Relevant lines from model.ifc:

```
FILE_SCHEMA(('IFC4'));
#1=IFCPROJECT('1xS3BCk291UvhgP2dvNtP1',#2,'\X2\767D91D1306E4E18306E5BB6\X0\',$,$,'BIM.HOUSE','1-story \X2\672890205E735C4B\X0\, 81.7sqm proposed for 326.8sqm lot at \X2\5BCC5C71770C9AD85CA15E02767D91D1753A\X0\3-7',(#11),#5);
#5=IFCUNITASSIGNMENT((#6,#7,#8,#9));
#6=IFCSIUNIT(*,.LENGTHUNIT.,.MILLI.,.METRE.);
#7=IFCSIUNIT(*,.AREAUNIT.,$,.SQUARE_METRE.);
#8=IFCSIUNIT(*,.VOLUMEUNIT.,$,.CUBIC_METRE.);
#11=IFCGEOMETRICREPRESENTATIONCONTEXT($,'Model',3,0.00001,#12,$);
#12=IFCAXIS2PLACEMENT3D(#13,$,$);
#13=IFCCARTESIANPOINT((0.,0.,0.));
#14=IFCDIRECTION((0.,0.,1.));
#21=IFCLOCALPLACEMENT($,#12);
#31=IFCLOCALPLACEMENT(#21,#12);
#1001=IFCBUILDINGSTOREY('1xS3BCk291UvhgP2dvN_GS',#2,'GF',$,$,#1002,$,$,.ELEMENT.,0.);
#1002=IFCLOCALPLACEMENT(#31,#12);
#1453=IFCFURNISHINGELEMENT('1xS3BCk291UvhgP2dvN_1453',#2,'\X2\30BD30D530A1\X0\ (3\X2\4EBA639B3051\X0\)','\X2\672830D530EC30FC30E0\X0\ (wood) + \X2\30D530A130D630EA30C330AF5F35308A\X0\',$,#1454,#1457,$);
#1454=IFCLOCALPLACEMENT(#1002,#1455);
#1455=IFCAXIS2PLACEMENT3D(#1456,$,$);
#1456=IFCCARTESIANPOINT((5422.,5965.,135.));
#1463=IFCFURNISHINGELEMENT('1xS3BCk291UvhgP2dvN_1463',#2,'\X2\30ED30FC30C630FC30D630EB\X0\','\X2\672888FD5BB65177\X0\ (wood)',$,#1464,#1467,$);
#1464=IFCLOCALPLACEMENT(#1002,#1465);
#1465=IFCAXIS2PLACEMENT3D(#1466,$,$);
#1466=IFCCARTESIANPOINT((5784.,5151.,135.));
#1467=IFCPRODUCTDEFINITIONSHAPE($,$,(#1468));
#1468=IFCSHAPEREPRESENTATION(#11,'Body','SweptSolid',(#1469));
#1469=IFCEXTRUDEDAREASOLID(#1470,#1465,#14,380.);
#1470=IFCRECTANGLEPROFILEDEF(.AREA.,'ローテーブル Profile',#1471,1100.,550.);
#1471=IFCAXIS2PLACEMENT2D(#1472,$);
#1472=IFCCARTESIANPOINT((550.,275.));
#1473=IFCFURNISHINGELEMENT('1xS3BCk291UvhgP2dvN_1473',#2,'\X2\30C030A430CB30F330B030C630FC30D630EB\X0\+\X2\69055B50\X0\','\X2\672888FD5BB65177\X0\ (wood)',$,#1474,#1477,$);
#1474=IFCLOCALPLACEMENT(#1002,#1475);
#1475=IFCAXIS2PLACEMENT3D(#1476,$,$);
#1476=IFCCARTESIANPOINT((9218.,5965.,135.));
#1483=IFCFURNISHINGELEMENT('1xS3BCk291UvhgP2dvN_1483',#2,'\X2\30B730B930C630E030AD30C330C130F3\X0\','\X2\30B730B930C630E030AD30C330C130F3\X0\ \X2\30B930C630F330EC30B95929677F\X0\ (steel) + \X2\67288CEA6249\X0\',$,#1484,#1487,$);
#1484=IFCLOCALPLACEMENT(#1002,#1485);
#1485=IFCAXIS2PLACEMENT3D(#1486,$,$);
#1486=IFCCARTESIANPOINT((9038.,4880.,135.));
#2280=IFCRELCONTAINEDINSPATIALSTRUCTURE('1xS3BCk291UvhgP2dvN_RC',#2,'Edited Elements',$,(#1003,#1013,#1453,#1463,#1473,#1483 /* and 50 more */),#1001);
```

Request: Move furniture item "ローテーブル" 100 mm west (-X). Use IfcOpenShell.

```python
import ifcopenshell
import ifcopenshell.api.geometry
import ifcopenshell.util.placement

model = ifcopenshell.open("model.ifc")

item = model.by_guid("1xS3BCk291UvhgP2dvN_1463")
matrix = ifcopenshell.util.placement.get_local_placement(item.ObjectPlacement)
matrix[0, 3] -= 100.0
ifcopenshell.api.geometry.edit_object_placement(model, product=item, matrix=matrix, is_si=False)

print(ifcopenshell.util.placement.get_local_placement(item.ObjectPlacement).round(3) + 0.0)

model.write("model-out.ifc")
```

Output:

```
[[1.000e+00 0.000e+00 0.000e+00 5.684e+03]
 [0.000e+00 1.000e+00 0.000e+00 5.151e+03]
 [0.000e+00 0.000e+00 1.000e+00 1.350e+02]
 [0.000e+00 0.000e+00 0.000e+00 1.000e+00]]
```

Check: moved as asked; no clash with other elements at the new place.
